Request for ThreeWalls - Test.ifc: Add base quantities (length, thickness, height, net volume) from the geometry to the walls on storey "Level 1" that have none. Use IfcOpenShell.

First a look at what the model holds.

```python
import ifcopenshell
import ifcopenshell.util.element
import ifcopenshell.util.unit

model = ifcopenshell.open("ThreeWalls - Test.ifc")
print(model.schema)
for unit_type in ("LENGTHUNIT", "AREAUNIT", "VOLUMEUNIT"):
    print(unit_type, ifcopenshell.util.unit.calculate_unit_scale(model, unit_type))
storey = next(s for s in model.by_type("IfcBuildingStorey") if s.Name == "Level 1")
walls = [e for e in ifcopenshell.util.element.get_decomposition(storey) if e.is_a("IfcWall")]
for e in sorted(walls, key=lambda e: e.id()):
    print(e.id(), e.is_a(), e.Name, list(ifcopenshell.util.element.get_psets(e, qtos_only=True)), sep=" | ")
```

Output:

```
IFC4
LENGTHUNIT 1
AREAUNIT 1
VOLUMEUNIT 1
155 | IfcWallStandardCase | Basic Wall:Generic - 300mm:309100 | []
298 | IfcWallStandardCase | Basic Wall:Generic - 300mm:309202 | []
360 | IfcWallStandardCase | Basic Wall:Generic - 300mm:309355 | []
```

```python
import ifcopenshell
import ifcopenshell.api.pset
import ifcopenshell.geom
import ifcopenshell.util.element
import ifcopenshell.util.shape
import ifcopenshell.util.unit

model = ifcopenshell.open("ThreeWalls - Test.ifc")
unit_scale = ifcopenshell.util.unit.calculate_unit_scale(model)
volume_scale = ifcopenshell.util.unit.calculate_unit_scale(model, "VOLUMEUNIT")
settings = ifcopenshell.geom.settings()

storey = next(s for s in model.by_type("IfcBuildingStorey") if s.Name == "Level 1")
walls = [e for e in ifcopenshell.util.element.get_decomposition(storey) if e.is_a("IfcWall")]

for e in sorted(walls, key=lambda e: e.id()):
    if ifcopenshell.util.element.get_psets(e, qtos_only=True, should_inherit=False):
        continue
    # Geometry comes back in metres, in the element's own axes.
    shape = ifcopenshell.geom.create_shape(settings, e)
    values = {
        "Length": ifcopenshell.util.shape.get_x(shape.geometry) / unit_scale,
        "Width": ifcopenshell.util.shape.get_y(shape.geometry) / unit_scale,
        "Height": ifcopenshell.util.shape.get_z(shape.geometry) / unit_scale,
        "NetVolume": ifcopenshell.util.shape.get_volume(shape.geometry) / volume_scale,
    }
    qto = ifcopenshell.api.pset.add_qto(model, product=e, name="Qto_WallBaseQuantities")
    ifcopenshell.api.pset.edit_qto(model, qto=qto, properties=values)
    print(e.id(), {k: round(v, 3) for k, v in values.items()})

model.write("ThreeWalls - Test_edited.ifc")
```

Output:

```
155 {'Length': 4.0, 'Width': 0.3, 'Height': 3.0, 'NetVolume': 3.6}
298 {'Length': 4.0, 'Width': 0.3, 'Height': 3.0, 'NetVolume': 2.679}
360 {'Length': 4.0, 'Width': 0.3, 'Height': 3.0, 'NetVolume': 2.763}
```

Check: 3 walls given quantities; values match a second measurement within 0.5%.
